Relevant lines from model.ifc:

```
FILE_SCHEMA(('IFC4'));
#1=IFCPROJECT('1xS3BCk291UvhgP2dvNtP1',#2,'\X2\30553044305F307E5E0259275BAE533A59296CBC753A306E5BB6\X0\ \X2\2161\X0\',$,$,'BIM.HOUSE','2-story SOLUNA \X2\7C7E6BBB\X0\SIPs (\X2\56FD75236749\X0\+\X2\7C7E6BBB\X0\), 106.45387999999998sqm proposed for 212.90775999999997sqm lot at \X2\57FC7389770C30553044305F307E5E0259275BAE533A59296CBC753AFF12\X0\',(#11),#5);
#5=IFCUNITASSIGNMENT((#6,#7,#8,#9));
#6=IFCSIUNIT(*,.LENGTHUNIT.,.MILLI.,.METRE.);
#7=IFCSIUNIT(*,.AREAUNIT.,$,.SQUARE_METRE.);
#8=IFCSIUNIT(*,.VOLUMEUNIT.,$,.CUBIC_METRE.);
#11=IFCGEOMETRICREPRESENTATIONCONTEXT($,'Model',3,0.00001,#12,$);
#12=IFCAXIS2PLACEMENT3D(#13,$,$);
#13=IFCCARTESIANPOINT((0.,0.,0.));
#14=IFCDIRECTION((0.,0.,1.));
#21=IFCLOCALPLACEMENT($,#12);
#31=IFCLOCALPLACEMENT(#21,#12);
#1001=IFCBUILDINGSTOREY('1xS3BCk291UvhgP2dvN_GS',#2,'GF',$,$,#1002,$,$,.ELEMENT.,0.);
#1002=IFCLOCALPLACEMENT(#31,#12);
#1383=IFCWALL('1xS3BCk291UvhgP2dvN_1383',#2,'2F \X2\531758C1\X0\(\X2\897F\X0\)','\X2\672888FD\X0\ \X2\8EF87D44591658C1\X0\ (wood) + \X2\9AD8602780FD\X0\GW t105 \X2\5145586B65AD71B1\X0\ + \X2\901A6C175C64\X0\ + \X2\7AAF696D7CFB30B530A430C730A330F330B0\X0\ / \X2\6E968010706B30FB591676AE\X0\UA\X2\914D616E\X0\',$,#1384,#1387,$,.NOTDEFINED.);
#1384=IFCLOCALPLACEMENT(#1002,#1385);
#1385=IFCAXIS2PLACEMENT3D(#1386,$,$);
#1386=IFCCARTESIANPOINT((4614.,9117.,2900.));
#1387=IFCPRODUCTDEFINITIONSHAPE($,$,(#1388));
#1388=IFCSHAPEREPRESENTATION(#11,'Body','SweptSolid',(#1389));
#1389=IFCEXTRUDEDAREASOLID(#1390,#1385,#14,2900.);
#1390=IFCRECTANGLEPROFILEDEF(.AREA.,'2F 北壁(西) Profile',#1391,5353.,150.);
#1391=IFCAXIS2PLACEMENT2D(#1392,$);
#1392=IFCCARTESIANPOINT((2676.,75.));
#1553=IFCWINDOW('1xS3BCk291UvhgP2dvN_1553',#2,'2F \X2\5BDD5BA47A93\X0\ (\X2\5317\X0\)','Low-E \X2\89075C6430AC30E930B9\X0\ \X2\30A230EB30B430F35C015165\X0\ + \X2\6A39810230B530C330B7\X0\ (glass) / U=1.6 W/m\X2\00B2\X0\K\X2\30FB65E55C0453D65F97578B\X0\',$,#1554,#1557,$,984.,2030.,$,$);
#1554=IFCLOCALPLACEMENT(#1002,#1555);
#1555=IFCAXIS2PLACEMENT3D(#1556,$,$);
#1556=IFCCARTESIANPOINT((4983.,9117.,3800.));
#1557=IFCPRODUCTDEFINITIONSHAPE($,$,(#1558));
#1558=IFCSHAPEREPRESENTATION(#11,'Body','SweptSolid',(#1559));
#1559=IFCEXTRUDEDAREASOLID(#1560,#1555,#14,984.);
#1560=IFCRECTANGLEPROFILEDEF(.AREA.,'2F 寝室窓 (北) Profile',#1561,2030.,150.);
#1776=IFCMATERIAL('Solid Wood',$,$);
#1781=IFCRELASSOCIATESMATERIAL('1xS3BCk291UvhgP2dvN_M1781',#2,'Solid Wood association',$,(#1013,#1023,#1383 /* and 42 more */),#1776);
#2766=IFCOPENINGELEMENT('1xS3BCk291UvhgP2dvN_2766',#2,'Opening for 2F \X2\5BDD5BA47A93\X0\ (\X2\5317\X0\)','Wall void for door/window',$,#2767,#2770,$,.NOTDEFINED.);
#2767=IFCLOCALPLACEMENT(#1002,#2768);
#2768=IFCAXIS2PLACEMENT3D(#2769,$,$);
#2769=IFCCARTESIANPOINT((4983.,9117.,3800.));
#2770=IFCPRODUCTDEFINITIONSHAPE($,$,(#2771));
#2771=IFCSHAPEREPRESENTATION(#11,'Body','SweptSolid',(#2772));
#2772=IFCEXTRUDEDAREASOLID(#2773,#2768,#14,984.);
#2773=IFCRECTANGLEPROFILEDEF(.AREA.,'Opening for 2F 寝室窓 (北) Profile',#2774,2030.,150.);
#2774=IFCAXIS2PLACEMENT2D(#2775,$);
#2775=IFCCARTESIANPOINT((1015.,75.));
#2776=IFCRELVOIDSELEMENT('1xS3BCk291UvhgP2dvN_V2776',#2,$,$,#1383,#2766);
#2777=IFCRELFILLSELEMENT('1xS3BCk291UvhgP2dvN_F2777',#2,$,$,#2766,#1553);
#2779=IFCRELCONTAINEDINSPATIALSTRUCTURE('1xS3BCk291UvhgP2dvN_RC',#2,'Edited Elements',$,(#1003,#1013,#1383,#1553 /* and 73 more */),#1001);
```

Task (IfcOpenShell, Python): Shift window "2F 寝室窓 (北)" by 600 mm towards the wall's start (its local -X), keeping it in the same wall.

```python
import ifcopenshell
import ifcopenshell.api.geometry
import ifcopenshell.util.placement
import ifcopenshell.util.unit

model = ifcopenshell.open("model.ifc")
unit_scale = ifcopenshell.util.unit.calculate_unit_scale(model)

window = model.by_guid("1xS3BCk291UvhgP2dvN_1553")
opening = window.FillsVoids[0].RelatingOpeningElement
wall = opening.VoidsElements[0].RelatingBuildingElement

wall_matrix = ifcopenshell.util.placement.get_local_placement(wall.ObjectPlacement)
shift = wall_matrix[:3, 0] * -0.6 / unit_scale
before = ifcopenshell.util.placement.get_local_placement(window.ObjectPlacement)[:3, 3].copy()

# The window is not placed relative to its opening, so move both.
for product in (opening, window):
    matrix = ifcopenshell.util.placement.get_local_placement(product.ObjectPlacement)
    matrix[:3, 3] += shift
    ifcopenshell.api.geometry.edit_object_placement(model, product=product, matrix=matrix, is_si=False)

after = ifcopenshell.util.placement.get_local_placement(window.ObjectPlacement)[:3, 3]
print("window moved by", (after - before).round(3) + 0.0)

model.write("model_edited.ifc")
```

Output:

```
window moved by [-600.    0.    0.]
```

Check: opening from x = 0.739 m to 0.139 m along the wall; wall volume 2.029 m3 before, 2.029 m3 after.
